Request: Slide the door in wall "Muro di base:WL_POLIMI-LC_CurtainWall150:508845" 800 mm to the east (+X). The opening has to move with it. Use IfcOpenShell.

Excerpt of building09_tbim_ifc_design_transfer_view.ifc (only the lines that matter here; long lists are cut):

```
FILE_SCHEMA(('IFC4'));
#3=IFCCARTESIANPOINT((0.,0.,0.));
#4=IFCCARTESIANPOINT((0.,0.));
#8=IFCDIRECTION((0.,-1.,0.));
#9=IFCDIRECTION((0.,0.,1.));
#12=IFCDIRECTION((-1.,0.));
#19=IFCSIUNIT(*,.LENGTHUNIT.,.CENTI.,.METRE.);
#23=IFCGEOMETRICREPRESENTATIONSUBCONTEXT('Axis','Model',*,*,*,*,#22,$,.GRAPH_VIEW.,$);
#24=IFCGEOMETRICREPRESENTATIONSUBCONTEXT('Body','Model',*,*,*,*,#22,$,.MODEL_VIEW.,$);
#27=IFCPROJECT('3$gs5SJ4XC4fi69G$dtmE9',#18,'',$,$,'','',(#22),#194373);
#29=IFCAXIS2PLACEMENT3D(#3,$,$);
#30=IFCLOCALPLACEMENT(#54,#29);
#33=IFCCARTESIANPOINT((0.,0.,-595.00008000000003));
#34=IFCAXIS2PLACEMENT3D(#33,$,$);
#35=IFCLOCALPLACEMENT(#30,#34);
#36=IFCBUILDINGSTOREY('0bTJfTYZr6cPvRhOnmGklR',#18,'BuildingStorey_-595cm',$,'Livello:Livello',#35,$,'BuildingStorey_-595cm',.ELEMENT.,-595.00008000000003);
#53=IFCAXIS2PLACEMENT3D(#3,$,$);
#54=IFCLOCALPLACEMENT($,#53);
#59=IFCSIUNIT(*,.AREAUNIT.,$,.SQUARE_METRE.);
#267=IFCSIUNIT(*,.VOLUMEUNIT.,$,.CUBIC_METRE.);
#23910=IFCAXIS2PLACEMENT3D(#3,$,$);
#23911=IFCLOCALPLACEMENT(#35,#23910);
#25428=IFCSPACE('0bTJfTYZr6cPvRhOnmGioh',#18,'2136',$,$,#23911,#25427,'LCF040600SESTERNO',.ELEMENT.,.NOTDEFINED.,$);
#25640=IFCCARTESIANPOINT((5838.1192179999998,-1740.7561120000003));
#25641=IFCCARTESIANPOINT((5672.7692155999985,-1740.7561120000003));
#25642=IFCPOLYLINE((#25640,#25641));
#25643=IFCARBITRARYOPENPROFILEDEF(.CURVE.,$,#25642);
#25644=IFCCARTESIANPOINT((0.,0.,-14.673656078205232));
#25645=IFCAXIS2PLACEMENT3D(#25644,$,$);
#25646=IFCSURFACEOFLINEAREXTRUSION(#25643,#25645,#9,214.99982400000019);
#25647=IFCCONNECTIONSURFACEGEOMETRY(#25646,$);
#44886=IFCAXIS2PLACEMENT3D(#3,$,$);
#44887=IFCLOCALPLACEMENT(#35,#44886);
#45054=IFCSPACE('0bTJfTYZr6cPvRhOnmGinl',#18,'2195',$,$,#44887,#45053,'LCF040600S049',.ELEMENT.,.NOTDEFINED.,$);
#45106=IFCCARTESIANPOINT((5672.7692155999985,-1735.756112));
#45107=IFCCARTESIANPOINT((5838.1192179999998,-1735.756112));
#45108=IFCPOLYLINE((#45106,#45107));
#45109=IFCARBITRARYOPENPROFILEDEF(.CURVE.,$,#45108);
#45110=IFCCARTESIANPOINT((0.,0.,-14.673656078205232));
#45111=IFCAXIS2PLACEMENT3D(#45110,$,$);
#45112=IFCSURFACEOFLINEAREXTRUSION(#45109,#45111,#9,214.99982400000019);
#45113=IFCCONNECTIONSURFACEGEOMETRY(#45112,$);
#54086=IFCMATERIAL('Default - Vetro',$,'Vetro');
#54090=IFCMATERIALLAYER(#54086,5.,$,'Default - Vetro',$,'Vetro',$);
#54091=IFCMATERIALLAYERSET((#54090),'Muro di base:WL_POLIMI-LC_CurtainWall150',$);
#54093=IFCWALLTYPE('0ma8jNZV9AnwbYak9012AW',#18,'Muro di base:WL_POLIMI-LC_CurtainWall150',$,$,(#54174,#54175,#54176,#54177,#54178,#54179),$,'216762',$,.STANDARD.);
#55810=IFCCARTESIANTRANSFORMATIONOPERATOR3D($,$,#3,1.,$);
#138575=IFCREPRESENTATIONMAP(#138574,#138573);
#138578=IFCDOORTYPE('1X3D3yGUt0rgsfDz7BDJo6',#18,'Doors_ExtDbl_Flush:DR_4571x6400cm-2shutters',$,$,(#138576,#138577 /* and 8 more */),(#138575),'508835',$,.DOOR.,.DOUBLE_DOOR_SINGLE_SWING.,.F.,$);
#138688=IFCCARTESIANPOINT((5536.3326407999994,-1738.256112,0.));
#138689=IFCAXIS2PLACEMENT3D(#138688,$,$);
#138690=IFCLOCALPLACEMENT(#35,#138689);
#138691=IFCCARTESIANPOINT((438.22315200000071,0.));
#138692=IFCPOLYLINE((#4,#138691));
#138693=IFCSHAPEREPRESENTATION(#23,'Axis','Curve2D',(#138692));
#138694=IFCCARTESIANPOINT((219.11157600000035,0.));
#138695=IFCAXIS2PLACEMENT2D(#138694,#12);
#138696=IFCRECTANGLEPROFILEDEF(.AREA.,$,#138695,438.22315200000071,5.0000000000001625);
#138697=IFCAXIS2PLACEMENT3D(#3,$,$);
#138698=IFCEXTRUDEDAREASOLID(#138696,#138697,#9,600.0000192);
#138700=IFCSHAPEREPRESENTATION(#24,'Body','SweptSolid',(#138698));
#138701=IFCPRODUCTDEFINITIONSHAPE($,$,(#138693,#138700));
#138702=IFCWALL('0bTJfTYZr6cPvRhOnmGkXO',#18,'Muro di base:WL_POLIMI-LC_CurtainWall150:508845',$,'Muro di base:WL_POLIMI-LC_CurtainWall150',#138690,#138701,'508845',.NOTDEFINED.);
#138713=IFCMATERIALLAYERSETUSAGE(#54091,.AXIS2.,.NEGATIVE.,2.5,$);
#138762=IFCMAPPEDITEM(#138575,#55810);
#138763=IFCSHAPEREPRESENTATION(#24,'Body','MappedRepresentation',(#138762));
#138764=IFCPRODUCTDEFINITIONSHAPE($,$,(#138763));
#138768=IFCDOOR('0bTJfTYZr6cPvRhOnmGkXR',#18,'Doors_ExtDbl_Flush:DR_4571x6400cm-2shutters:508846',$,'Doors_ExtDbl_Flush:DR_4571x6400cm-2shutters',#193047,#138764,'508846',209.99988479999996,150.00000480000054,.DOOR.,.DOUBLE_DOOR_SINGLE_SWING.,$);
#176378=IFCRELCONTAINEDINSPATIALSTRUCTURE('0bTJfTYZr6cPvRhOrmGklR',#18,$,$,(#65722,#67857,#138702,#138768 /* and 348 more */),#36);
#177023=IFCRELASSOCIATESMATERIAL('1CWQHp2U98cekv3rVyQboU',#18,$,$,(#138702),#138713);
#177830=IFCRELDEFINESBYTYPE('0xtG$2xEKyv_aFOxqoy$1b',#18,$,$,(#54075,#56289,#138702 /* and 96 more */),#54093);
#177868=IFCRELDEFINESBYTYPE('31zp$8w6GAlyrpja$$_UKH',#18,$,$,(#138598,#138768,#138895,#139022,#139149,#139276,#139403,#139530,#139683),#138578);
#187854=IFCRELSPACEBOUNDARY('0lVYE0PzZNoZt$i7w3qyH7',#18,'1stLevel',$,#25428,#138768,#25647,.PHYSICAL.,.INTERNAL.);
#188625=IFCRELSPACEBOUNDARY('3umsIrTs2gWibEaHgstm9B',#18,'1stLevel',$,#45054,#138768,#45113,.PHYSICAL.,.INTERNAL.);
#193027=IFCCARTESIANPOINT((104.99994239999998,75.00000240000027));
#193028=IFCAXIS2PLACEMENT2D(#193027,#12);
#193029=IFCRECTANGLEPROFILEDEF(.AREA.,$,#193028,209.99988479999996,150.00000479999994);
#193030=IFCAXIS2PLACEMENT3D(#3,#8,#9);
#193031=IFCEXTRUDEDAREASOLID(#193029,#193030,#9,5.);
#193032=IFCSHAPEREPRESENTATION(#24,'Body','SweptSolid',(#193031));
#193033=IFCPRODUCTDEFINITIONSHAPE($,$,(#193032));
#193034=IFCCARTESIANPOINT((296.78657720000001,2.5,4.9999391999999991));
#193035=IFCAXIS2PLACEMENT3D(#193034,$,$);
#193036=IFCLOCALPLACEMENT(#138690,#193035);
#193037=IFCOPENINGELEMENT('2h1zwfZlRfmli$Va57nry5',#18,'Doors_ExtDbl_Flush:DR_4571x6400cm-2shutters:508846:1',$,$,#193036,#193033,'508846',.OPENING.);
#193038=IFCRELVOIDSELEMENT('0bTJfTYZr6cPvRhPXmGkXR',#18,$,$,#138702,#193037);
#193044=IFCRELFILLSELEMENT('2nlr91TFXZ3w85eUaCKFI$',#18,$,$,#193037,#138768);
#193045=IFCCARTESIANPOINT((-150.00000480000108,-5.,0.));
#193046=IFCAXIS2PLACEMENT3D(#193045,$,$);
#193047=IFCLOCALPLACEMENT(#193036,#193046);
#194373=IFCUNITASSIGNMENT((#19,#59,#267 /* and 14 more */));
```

```python
import numpy as np
import ifcopenshell
import ifcopenshell.api.geometry
import ifcopenshell.util.placement
import ifcopenshell.util.unit

model = ifcopenshell.open("building09_tbim_ifc_design_transfer_view.ifc")
unit_scale = ifcopenshell.util.unit.calculate_unit_scale(model)

door = model.by_guid("0bTJfTYZr6cPvRhOnmGkXR")
opening = door.FillsVoids[0].RelatingOpeningElement
wall = opening.VoidsElements[0].RelatingBuildingElement

wall_matrix = ifcopenshell.util.placement.get_local_placement(wall.ObjectPlacement)
shift = wall_matrix[:3, 0] * 0.8 / unit_scale
before = ifcopenshell.util.placement.get_local_placement(door.ObjectPlacement)[:3, 3].copy()

# The door is placed relative to its opening, so it follows when the opening moves.
matrix = ifcopenshell.util.placement.get_local_placement(opening.ObjectPlacement)
matrix[:3, 3] += shift
ifcopenshell.api.geometry.edit_object_placement(
    model, product=opening, matrix=matrix, is_si=False, should_transform_children=True
)

# Space boundary surfaces are stored in each space's coordinates; move them too.
for rel in door.ProvidesBoundaries:
    if not rel.ConnectionGeometry:
        continue
    surface = rel.ConnectionGeometry.SurfaceOnRelatingElement
    space_matrix = ifcopenshell.util.placement.get_local_placement(rel.RelatingSpace.ObjectPlacement)
    point = np.array(surface.Position.Location.Coordinates) + space_matrix[:3, :3].T @ shift
    surface.Position = model.createIfcAxis2Placement3D(
        model.createIfcCartesianPoint(point.tolist()), surface.Position.Axis, surface.Position.RefDirection
    )

after = ifcopenshell.util.placement.get_local_placement(door.ObjectPlacement)[:3, 3]
print("door moved by", (after - before).round(3) + 0.0)

model.write("building09_tbim_ifc_design_transfer_view-out.ifc")
```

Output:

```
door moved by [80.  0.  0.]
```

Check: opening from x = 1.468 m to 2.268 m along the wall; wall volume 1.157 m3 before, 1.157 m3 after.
